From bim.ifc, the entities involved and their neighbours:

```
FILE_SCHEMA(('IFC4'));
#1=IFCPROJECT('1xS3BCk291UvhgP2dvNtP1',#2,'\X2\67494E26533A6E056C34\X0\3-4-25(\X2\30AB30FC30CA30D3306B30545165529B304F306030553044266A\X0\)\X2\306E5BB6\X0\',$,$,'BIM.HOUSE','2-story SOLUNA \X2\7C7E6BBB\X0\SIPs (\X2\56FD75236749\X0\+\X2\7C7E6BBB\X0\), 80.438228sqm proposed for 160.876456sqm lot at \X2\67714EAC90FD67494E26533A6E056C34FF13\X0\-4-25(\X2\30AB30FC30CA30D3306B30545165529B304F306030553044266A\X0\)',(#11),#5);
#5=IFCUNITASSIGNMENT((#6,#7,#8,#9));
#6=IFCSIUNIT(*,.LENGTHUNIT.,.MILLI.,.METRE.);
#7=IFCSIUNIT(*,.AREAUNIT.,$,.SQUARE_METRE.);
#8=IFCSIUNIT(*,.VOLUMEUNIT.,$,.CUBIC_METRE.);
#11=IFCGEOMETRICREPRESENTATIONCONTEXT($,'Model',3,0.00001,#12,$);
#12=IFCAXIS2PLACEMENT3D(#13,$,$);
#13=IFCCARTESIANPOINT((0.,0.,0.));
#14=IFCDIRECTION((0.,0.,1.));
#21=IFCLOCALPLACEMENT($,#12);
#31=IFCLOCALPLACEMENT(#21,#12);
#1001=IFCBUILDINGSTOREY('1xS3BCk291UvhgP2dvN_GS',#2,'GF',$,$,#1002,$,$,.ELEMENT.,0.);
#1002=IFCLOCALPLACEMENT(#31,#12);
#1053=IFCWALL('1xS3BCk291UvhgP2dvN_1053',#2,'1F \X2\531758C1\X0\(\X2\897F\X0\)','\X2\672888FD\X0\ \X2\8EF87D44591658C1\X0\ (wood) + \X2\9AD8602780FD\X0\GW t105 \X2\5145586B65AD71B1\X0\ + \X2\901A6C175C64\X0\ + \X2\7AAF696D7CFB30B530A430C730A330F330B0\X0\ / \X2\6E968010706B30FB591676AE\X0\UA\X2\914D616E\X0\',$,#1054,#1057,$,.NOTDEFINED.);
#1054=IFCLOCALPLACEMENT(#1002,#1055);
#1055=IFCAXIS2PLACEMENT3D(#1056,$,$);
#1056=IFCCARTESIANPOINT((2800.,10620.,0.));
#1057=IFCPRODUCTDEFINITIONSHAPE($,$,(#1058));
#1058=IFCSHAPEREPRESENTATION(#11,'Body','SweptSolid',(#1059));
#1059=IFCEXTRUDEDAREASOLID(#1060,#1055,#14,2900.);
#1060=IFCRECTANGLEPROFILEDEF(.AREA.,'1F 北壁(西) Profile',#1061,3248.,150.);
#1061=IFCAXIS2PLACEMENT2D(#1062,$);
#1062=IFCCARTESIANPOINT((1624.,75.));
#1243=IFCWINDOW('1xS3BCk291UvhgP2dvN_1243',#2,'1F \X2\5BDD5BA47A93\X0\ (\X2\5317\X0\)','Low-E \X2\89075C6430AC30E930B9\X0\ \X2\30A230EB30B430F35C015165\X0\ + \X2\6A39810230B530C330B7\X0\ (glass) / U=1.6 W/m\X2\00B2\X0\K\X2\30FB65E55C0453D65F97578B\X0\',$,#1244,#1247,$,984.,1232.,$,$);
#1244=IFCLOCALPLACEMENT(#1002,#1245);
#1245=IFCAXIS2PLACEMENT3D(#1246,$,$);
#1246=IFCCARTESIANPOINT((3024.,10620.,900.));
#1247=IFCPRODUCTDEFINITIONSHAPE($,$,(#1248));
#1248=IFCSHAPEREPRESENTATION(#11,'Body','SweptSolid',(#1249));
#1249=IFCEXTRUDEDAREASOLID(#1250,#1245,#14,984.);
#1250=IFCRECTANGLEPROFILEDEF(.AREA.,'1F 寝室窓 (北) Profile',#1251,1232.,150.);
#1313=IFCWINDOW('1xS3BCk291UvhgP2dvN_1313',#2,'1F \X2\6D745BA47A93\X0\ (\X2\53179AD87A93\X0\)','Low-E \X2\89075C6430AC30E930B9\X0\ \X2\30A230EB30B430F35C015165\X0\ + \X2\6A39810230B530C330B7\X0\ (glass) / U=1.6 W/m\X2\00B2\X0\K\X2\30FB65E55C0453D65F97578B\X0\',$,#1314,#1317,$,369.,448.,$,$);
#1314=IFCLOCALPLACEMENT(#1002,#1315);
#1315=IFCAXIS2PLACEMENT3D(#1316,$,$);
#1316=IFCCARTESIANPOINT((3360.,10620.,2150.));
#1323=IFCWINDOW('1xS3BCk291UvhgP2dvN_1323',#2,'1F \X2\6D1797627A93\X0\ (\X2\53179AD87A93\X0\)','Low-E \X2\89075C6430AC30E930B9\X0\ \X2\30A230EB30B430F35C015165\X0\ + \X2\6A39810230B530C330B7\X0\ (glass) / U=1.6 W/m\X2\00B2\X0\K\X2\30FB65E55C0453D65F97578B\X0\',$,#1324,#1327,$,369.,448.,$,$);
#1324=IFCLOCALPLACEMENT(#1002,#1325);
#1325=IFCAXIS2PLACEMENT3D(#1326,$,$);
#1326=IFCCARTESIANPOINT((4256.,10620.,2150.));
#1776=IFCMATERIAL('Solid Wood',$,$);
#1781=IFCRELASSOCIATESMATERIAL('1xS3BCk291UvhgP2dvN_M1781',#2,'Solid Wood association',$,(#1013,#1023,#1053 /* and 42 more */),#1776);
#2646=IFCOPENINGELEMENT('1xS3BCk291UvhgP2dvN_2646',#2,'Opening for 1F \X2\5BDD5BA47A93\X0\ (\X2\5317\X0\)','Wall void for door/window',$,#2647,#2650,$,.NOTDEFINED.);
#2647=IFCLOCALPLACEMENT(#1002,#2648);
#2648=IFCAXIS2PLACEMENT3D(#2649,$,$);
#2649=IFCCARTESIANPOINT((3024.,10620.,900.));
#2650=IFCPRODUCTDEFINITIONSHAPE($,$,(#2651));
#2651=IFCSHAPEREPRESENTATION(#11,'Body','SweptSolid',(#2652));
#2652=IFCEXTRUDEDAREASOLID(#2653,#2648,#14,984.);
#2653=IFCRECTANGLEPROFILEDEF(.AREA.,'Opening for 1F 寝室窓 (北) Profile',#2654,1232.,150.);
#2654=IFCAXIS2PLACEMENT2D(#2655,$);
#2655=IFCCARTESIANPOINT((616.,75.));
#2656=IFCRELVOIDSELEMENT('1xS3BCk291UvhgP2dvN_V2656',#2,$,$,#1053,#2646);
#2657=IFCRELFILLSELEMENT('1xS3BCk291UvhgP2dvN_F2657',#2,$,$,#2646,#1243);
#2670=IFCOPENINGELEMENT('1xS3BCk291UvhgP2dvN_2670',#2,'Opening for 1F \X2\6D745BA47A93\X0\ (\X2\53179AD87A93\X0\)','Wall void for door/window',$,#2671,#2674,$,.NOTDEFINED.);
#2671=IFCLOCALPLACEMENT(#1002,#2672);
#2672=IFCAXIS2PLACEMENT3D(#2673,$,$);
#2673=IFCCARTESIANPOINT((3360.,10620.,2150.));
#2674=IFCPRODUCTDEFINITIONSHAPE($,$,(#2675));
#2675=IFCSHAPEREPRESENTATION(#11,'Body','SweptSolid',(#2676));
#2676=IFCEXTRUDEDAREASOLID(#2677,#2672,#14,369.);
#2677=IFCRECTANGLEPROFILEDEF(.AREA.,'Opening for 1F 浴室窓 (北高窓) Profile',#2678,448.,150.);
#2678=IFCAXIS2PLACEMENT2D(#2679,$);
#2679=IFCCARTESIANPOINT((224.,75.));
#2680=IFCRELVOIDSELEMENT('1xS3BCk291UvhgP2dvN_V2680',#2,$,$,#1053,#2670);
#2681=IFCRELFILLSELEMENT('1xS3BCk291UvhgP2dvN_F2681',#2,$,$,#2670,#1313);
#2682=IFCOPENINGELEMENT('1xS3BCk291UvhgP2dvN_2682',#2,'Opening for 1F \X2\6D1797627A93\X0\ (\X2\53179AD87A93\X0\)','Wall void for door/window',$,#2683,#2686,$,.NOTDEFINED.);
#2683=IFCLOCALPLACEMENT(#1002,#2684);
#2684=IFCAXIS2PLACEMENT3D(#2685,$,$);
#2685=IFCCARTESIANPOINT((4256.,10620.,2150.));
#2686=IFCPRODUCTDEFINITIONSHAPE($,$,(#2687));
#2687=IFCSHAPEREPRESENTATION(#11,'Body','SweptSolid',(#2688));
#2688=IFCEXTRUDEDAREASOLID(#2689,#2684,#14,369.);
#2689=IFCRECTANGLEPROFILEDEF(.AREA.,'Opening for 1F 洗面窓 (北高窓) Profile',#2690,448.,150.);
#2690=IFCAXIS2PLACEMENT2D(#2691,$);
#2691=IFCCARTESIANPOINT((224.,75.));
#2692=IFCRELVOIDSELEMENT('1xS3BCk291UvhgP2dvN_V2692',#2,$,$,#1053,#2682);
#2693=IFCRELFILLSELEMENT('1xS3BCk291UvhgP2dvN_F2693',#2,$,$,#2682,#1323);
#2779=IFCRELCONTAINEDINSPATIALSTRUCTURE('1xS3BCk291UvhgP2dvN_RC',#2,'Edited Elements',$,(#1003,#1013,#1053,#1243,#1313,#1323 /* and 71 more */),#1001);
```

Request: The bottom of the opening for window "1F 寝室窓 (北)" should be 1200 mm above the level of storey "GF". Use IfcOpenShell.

```python
import numpy as np
import ifcopenshell
import ifcopenshell.api.geometry
import ifcopenshell.geom
import ifcopenshell.util.element
import ifcopenshell.util.placement
import ifcopenshell.util.shape
import ifcopenshell.util.unit

model = ifcopenshell.open("bim.ifc")
unit_scale = ifcopenshell.util.unit.calculate_unit_scale(model)

window = model.by_guid("1xS3BCk291UvhgP2dvN_1243")
opening = window.FillsVoids[0].RelatingOpeningElement
storey = ifcopenshell.util.element.get_container(window, ifc_class="IfcBuildingStorey")
level = ifcopenshell.util.placement.get_local_placement(storey.ObjectPlacement)[2, 3]

# The opening's origin need not be at the sill, so measure its lowest point.
shape = ifcopenshell.geom.create_shape(ifcopenshell.geom.settings(), opening)
bottom = ifcopenshell.util.shape.get_shape_bottom_elevation(shape, shape.geometry) / unit_scale
dz = level + 1200.0 - bottom

shift = np.array([0.0, 0.0, dz])
# The window is not placed relative to its opening, so move both.
for product in (opening, window):
    matrix = ifcopenshell.util.placement.get_local_placement(product.ObjectPlacement)
    matrix[:3, 3] += shift
    ifcopenshell.api.geometry.edit_object_placement(model, product=product, matrix=matrix, is_si=False)

print(f"moved by {dz * unit_scale:+.3f} m")

model.write("bim_rev.ifc")
```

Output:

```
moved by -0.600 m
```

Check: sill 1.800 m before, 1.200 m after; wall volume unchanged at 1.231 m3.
